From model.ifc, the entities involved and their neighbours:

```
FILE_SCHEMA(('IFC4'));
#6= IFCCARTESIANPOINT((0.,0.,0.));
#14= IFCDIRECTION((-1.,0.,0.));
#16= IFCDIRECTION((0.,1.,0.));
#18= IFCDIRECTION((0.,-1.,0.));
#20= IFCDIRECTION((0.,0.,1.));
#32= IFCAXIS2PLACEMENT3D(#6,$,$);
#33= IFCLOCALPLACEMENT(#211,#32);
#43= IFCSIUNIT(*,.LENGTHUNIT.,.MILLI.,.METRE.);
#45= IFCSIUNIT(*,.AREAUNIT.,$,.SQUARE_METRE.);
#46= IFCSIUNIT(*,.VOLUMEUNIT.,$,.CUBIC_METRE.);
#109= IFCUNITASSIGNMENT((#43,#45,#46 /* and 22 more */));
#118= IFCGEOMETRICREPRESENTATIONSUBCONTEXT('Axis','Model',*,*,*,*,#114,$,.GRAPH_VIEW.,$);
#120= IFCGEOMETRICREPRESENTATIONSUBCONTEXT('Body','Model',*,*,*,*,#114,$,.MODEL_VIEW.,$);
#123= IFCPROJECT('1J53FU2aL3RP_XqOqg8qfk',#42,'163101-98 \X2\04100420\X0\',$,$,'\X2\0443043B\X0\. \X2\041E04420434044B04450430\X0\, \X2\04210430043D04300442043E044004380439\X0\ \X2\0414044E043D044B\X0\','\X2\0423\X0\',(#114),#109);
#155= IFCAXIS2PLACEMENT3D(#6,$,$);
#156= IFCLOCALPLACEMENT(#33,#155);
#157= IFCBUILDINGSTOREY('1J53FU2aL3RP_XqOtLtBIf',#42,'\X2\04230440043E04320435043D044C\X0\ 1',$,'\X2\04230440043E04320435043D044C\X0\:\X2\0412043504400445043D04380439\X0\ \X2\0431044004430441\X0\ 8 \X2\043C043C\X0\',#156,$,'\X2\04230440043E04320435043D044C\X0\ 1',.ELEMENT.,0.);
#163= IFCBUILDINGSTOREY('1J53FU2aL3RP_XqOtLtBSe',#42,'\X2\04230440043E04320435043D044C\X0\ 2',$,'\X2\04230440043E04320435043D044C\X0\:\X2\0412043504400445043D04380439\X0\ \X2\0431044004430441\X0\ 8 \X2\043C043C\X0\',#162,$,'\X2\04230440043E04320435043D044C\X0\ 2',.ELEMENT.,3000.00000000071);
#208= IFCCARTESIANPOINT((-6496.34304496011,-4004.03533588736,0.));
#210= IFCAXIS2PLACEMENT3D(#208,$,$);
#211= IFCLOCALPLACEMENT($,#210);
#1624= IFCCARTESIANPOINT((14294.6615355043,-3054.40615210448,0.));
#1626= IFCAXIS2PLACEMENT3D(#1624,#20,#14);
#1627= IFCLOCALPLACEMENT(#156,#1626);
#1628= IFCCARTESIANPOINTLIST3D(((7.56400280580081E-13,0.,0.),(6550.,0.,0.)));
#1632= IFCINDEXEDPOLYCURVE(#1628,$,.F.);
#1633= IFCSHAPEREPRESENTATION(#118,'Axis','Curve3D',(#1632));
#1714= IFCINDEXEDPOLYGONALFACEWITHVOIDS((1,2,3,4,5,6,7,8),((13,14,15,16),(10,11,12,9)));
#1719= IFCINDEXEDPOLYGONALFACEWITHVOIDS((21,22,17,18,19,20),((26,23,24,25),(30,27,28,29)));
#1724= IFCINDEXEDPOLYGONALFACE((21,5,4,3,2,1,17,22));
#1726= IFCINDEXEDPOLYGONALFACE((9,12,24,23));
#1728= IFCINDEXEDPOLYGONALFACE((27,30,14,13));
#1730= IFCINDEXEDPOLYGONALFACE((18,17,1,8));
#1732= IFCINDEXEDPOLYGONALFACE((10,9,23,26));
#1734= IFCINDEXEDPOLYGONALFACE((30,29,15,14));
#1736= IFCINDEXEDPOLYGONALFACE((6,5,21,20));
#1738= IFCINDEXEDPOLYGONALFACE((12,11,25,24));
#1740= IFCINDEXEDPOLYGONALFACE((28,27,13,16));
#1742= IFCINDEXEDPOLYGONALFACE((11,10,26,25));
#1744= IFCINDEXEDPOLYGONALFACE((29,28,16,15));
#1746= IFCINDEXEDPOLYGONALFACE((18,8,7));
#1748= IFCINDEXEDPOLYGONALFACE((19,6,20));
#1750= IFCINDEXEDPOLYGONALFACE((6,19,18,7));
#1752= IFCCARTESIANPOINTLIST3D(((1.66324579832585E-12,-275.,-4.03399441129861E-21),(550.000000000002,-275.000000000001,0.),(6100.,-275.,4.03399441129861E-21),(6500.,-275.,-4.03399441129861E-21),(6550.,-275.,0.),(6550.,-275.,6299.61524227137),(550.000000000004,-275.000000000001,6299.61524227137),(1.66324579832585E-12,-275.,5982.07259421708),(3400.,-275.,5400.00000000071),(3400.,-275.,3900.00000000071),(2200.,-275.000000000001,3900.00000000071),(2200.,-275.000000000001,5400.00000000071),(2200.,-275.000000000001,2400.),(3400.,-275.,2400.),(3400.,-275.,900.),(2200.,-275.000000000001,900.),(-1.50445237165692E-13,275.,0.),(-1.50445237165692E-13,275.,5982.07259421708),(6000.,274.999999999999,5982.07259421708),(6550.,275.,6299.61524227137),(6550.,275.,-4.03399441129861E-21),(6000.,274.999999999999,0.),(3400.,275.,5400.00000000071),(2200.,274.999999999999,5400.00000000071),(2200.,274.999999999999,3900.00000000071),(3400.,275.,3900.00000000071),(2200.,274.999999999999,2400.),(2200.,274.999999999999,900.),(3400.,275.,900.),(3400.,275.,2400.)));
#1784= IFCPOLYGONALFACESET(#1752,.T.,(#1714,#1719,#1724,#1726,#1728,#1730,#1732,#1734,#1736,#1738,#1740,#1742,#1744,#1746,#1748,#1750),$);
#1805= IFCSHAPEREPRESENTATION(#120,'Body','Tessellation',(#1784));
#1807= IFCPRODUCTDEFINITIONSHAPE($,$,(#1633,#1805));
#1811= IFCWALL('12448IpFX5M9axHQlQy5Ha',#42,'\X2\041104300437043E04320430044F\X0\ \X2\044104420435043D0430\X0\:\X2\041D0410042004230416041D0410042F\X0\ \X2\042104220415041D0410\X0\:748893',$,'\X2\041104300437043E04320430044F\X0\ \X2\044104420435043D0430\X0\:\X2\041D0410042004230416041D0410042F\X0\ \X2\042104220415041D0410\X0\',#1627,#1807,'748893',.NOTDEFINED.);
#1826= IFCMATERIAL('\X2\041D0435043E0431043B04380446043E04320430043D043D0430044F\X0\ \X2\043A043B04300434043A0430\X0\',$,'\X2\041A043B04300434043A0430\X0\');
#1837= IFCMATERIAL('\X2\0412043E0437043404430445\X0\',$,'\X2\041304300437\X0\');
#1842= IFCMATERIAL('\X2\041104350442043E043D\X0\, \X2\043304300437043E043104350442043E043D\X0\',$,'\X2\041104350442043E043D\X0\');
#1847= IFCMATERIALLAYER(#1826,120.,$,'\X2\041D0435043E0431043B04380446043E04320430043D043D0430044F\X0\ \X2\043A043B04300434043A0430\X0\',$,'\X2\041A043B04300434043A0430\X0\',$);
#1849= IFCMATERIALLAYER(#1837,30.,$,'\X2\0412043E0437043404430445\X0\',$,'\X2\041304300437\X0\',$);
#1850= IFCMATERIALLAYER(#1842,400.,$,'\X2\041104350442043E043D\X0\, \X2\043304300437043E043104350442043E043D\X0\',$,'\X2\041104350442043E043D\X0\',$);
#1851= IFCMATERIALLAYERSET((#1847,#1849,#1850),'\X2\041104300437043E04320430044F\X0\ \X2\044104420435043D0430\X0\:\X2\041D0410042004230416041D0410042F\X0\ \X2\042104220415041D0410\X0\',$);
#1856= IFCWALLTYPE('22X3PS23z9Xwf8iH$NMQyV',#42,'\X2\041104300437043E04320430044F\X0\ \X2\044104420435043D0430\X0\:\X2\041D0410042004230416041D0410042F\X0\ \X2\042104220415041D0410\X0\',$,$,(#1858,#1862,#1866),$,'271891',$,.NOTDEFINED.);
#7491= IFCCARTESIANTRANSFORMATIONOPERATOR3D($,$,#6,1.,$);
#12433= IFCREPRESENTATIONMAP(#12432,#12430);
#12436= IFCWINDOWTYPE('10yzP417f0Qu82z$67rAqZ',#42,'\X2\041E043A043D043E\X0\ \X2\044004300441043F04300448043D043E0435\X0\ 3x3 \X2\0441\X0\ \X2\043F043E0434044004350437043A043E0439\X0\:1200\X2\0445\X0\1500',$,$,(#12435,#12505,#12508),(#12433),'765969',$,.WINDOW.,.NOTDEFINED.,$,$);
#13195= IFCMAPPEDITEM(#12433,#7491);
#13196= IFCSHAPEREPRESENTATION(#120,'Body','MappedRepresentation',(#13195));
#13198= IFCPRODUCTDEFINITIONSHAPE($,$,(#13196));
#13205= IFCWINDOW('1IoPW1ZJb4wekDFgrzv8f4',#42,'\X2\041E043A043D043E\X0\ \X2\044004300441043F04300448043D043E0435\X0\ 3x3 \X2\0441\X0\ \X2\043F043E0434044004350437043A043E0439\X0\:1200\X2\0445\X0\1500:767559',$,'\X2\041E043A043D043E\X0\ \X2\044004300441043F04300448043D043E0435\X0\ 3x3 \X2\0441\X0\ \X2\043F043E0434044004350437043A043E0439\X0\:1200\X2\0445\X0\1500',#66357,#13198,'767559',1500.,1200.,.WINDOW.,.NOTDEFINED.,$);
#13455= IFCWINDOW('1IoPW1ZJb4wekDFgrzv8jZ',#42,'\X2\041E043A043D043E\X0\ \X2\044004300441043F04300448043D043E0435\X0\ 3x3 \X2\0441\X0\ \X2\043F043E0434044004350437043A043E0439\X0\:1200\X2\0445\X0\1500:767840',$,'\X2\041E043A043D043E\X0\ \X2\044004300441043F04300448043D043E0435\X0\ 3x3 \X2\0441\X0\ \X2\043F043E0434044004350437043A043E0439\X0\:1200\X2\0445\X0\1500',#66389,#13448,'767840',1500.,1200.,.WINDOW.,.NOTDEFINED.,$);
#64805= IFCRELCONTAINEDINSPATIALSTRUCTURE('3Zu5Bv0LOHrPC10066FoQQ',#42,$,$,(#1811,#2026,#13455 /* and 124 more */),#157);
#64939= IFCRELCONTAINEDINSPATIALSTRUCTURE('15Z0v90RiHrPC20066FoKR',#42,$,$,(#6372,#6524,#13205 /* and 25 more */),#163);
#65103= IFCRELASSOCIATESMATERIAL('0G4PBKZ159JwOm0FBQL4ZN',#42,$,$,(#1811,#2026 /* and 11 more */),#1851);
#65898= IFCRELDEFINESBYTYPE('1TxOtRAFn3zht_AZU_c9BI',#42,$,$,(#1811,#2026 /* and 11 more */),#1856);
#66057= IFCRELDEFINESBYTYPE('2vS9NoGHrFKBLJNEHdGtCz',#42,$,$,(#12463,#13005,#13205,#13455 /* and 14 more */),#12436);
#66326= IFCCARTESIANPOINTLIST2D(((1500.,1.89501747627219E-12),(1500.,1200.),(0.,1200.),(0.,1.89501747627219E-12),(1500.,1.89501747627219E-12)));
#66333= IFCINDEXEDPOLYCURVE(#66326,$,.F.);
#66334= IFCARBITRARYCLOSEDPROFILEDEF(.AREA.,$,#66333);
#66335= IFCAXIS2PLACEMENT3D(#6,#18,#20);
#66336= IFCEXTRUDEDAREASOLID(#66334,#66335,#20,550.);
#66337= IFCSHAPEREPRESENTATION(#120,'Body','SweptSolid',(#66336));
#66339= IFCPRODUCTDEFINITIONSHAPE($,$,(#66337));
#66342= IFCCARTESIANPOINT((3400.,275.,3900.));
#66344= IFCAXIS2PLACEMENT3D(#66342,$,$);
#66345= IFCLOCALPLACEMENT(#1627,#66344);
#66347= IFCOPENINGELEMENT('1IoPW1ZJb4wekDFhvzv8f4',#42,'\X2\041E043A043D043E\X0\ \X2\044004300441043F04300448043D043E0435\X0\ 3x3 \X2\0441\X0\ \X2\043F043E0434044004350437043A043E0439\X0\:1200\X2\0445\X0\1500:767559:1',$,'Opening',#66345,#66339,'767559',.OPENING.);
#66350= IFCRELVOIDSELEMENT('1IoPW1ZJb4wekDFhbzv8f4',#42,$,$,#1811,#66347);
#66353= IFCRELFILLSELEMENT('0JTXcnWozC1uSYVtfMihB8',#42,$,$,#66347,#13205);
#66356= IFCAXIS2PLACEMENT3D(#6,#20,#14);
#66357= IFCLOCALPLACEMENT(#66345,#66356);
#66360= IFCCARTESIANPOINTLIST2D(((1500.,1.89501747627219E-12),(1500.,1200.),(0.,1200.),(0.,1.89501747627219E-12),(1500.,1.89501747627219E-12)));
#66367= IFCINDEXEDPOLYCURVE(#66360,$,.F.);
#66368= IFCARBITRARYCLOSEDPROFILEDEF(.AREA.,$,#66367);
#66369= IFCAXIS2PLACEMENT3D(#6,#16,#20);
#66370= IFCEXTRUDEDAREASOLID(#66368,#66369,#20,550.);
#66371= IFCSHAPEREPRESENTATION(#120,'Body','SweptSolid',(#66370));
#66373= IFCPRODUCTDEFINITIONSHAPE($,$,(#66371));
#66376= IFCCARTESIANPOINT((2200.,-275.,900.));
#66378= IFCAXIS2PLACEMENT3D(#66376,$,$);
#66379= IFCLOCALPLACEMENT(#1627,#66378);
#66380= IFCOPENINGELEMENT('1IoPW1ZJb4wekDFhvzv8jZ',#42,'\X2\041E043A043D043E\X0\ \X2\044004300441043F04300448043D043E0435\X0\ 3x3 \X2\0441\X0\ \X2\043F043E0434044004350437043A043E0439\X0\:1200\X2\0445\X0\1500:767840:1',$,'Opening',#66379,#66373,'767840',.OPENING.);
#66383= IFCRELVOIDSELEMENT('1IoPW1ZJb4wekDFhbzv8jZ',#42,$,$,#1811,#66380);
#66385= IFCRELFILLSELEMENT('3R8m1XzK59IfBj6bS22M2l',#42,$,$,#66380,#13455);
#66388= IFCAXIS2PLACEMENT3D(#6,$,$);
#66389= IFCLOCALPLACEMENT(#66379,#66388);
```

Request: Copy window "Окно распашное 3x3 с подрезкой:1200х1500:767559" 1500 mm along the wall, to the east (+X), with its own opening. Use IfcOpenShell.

```python
import ifcopenshell
import ifcopenshell.api.feature
import ifcopenshell.api.geometry
import ifcopenshell.api.root
import ifcopenshell.geom
import ifcopenshell.util.element
import ifcopenshell.util.placement
import ifcopenshell.util.shape

model = ifcopenshell.open("model.ifc")
settings = ifcopenshell.geom.settings()


def volume(element):
    """Net volume in cubic metres, openings subtracted."""
    shape = ifcopenshell.geom.create_shape(settings, element)
    return ifcopenshell.util.shape.get_volume(shape.geometry)


def reuse_history(source, copy):
    """copy_class also copies each property set's owner history, people and application; keep the originals."""
    for rel in copy.IsDefinedBy:
        if rel.is_a("IfcRelDefinesByProperties") and (history := rel.RelatingPropertyDefinition.OwnerHistory):
            rel.RelatingPropertyDefinition.OwnerHistory = source.OwnerHistory
            ifcopenshell.util.element.remove_deep2(model, history)


window = model.by_id(13205)
opening = window.FillsVoids[0].RelatingOpeningElement
wall = opening.VoidsElements[0].RelatingBuildingElement
before = volume(wall)
shift = ifcopenshell.util.placement.get_local_placement(wall.ObjectPlacement)[:3, 0] * -1500.0

# copy_class copies the void relationship, type, container and properties, but no geometry.
new_opening = ifcopenshell.api.root.copy_class(model, product=opening)
new_opening.Representation = ifcopenshell.util.element.copy_deep(
    model, opening.Representation, exclude=["IfcGeometricRepresentationContext", "IfcRepresentationMap"]
)
new_opening.Name = "Окно распашное 3x3 с подрезкой:1200х1500"
new_opening.Tag = None
new_window = ifcopenshell.api.root.copy_class(model, product=window)
new_window.Representation = ifcopenshell.util.element.copy_deep(
    model, window.Representation, exclude=["IfcGeometricRepresentationContext", "IfcRepresentationMap"]
)
new_window.Name = "Окно распашное 3x3 с подрезкой:1200х1500"
new_window.Tag = None
reuse_history(window, new_window)
ifcopenshell.api.feature.add_filling(model, opening=new_opening, element=new_window)

for old, new in ((opening, new_opening), (window, new_window)):
    matrix = ifcopenshell.util.placement.get_local_placement(old.ObjectPlacement)
    matrix[:3, 3] += shift
    ifcopenshell.api.geometry.edit_object_placement(model, product=new, matrix=matrix, is_si=False)

after = volume(wall)

print(f"wall volume {before:.3f} -> {after:.3f} m3")

model.write("model-out.ifc")
```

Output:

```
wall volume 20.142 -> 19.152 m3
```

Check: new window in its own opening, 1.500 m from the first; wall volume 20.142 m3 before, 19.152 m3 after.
